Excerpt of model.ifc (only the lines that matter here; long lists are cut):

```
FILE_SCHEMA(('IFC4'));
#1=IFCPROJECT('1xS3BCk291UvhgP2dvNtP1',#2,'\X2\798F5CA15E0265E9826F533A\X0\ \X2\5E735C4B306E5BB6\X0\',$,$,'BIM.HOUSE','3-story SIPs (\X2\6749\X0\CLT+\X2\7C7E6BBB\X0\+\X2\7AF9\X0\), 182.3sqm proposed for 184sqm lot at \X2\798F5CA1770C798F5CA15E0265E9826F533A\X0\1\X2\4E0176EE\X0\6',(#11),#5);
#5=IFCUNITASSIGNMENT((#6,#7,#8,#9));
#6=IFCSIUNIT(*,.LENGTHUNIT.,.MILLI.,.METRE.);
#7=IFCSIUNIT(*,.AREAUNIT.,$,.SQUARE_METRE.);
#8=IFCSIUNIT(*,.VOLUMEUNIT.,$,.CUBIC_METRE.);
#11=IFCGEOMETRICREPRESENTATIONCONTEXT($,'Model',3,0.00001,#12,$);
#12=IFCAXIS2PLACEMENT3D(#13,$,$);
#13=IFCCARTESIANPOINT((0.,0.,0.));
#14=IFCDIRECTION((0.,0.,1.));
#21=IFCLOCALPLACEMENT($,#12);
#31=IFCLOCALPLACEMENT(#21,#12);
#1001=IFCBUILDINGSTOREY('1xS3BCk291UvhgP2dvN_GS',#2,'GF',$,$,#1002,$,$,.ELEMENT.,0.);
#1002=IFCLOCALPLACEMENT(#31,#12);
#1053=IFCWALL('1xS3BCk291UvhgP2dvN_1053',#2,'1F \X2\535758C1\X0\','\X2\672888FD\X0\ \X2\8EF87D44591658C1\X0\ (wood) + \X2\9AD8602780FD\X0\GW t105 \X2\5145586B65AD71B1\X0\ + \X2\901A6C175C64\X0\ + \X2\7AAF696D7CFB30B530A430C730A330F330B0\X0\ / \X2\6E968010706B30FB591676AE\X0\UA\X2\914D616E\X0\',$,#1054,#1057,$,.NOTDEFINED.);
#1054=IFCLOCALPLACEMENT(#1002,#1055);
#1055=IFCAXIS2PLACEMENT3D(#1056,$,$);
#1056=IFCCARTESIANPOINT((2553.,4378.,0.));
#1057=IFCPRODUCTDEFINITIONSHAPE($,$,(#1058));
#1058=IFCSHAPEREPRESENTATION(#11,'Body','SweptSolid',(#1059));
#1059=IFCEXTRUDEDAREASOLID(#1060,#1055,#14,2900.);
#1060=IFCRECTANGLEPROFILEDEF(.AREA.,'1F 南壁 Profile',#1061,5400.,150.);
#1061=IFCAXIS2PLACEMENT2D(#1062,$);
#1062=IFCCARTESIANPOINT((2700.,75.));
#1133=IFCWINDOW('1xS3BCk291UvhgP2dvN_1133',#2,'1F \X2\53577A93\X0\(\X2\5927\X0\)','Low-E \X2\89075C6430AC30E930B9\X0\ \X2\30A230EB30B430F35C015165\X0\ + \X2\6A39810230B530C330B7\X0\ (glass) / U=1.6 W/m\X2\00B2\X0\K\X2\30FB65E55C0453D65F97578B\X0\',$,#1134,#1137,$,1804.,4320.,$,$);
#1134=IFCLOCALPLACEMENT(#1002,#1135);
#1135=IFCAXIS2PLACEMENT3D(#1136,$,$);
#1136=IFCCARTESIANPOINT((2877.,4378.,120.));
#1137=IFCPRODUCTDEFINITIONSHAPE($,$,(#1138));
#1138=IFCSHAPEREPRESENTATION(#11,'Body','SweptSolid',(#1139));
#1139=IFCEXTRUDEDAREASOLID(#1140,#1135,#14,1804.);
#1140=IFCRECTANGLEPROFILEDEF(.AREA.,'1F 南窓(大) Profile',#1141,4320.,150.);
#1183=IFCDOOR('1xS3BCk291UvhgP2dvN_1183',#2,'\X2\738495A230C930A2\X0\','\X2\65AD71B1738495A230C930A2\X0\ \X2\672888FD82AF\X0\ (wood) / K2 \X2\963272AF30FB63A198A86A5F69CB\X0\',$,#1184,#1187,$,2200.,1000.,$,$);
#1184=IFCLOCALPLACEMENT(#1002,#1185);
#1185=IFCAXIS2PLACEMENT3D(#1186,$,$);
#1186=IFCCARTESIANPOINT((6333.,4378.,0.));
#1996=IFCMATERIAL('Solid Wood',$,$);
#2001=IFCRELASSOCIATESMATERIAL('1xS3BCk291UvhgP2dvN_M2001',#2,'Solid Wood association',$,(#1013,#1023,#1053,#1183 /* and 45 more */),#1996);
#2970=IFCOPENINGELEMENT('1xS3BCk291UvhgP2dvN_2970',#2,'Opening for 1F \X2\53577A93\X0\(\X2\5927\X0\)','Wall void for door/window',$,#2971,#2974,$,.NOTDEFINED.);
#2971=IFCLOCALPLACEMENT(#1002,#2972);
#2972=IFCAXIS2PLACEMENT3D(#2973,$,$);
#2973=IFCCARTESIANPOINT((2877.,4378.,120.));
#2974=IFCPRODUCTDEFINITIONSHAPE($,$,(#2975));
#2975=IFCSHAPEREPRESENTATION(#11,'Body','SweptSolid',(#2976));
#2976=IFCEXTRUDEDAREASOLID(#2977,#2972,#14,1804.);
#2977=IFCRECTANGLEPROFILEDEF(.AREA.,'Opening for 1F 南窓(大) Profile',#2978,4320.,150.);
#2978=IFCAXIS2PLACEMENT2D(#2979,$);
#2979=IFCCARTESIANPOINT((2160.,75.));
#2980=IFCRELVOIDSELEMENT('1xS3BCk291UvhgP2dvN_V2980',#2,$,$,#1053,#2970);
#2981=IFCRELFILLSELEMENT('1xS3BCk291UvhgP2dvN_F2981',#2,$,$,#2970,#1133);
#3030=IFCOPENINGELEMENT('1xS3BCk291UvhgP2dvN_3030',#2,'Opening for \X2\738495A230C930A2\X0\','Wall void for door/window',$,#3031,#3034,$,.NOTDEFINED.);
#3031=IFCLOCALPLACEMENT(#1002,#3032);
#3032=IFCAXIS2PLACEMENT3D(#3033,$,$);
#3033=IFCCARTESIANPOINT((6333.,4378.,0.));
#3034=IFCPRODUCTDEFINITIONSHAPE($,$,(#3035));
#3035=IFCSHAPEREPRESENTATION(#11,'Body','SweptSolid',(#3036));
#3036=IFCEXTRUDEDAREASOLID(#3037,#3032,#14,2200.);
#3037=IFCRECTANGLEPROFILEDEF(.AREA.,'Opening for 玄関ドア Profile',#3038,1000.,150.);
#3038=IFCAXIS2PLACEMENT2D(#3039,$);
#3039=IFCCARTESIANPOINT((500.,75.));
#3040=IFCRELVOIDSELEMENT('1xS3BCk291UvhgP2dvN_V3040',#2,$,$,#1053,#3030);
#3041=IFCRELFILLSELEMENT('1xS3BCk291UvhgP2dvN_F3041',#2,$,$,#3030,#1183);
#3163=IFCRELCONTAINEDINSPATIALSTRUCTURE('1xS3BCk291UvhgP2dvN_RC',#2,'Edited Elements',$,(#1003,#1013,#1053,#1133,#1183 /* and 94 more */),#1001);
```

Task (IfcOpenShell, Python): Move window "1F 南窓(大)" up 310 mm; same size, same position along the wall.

```python
import numpy as np
import ifcopenshell
import ifcopenshell.api.geometry
import ifcopenshell.util.placement
import ifcopenshell.util.unit

model = ifcopenshell.open("model.ifc")
unit_scale = ifcopenshell.util.unit.calculate_unit_scale(model)

window = model.by_guid("1xS3BCk291UvhgP2dvN_1133")
opening = window.FillsVoids[0].RelatingOpeningElement
dz = 0.31 / unit_scale

shift = np.array([0.0, 0.0, dz])
# The window is not placed relative to its opening, so move both.
for product in (opening, window):
    matrix = ifcopenshell.util.placement.get_local_placement(product.ObjectPlacement)
    matrix[:3, 3] += shift
    ifcopenshell.api.geometry.edit_object_placement(model, product=product, matrix=matrix, is_si=False)

print(f"moved by {dz * unit_scale:+.3f} m")

model.write("model_v2.ifc")
```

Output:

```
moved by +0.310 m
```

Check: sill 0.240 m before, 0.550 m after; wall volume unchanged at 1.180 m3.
